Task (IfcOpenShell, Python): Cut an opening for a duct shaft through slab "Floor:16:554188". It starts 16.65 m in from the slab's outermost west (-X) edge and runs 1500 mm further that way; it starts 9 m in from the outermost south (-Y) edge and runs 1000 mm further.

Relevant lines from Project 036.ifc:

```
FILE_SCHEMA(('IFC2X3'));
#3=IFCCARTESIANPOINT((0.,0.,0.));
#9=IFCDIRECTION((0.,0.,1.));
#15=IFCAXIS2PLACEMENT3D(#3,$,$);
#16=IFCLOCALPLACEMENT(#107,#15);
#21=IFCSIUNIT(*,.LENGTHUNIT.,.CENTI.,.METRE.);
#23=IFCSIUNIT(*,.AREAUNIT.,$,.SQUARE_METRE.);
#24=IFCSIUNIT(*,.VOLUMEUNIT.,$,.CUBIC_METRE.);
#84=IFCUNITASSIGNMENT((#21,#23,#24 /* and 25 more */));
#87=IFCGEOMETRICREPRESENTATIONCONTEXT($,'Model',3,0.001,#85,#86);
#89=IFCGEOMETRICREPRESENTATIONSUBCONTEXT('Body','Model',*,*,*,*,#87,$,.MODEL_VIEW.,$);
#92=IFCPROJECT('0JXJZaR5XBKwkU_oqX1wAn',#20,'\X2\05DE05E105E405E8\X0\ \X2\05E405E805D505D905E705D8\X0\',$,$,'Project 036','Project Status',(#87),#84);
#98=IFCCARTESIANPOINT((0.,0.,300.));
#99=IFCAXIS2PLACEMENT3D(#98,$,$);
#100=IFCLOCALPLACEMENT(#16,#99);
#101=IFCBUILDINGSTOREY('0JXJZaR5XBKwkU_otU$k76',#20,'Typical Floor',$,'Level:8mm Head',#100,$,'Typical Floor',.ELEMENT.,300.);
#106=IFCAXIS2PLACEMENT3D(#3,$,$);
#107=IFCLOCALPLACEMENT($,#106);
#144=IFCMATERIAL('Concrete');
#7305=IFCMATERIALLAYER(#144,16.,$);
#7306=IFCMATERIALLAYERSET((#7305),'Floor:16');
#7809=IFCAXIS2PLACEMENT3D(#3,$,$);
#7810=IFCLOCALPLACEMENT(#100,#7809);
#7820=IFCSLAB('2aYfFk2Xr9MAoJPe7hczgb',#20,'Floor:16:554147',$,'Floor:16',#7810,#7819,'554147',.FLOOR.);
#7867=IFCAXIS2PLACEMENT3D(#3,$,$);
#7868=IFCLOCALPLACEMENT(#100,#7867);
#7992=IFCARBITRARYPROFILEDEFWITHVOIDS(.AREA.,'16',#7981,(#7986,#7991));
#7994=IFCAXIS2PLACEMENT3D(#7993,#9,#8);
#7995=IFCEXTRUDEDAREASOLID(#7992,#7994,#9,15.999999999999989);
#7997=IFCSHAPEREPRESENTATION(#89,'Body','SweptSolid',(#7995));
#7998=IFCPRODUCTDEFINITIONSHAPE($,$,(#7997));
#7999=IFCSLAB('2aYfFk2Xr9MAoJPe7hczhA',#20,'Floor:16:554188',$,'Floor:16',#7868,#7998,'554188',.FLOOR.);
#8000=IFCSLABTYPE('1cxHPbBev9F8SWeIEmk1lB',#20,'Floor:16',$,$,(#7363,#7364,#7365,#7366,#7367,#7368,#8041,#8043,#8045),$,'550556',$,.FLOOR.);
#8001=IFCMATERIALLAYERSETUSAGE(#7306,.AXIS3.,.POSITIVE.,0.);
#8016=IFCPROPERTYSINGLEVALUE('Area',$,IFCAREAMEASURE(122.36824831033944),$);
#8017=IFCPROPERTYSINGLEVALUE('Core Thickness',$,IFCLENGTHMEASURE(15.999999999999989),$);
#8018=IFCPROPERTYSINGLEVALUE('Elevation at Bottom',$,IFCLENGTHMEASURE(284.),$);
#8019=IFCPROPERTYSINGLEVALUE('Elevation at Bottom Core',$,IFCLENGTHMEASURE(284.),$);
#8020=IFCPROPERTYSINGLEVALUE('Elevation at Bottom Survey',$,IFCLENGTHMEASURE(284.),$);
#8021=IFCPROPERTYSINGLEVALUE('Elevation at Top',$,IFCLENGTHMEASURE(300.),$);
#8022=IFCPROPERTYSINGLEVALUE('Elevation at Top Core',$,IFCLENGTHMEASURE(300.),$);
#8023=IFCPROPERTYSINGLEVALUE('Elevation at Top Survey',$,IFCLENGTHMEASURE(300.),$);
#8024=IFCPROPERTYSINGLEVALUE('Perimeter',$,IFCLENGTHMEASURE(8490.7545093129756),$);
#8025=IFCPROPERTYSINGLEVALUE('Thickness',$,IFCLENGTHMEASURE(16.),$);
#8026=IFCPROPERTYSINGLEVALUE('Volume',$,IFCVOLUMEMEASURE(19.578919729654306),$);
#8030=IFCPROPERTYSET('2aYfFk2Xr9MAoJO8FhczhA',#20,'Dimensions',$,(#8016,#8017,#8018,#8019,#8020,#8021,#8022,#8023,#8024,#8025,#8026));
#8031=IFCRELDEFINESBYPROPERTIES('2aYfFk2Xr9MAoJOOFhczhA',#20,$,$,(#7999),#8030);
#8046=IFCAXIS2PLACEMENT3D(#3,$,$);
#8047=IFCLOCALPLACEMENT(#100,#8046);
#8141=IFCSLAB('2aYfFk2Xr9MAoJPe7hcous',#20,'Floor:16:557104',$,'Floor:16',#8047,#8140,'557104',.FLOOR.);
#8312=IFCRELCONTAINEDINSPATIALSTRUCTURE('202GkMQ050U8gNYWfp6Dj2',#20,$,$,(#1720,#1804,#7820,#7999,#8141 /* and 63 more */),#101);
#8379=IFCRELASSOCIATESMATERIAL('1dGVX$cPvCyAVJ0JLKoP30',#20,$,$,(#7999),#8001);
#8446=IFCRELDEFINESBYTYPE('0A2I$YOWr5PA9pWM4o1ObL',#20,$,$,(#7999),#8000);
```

```python
import numpy as np
import ifcopenshell
import ifcopenshell.api.feature
import ifcopenshell.api.geometry
import ifcopenshell.api.pset
import ifcopenshell.api.root
import ifcopenshell.geom
import ifcopenshell.util.element
import ifcopenshell.util.placement
import ifcopenshell.util.representation
import ifcopenshell.util.shape
import ifcopenshell.util.unit

model = ifcopenshell.open("Project 036.ifc")
unit_scale = ifcopenshell.util.unit.calculate_unit_scale(model)
area_scale = ifcopenshell.util.unit.calculate_unit_scale(model, "AREAUNIT")
volume_scale = ifcopenshell.util.unit.calculate_unit_scale(model, "VOLUMEUNIT")
settings = ifcopenshell.geom.settings()


def volume(element):
    """Net volume in cubic metres, openings subtracted."""
    shape = ifcopenshell.geom.create_shape(settings, element)
    return ifcopenshell.util.shape.get_volume(shape.geometry)


slab = model.by_guid("2aYfFk2Xr9MAoJPe7hczhA")
before = volume(slab)

# Extent in the slab's own axes, in metres. The edges named are its -X and -Y sides.
slab_shape = ifcopenshell.geom.create_shape(settings, slab)
vertices = ifcopenshell.util.shape.get_vertices(slab_shape.geometry)
x_min, y_min, bottom = vertices.min(axis=0)
top = vertices[:, 2].max()

opening = ifcopenshell.api.root.create_entity(model, ifc_class="IfcOpeningElement", name="Duct shaft opening")
context = ifcopenshell.util.representation.get_context(model, "Model", "Body", "MODEL_VIEW")
width, depth = 1.5, 1
outline = [(0.0, 0.0), (width, 0.0), (width, depth), (0.0, depth), (0.0, 0.0)]
# Overshoot both faces by 50 mm so the cut is clean.
shape = ifcopenshell.api.geometry.add_slab_representation(
    model, context=context, depth=top - bottom + 0.1, polyline=outline
)
ifcopenshell.api.geometry.assign_representation(model, product=opening, representation=shape)

matrix = ifcopenshell.util.placement.get_local_placement(slab.ObjectPlacement)
matrix[:, 3] = matrix @ np.append(np.array([x_min + 16.65, y_min + 9, bottom - 0.05]) / unit_scale, 1.0)
ifcopenshell.api.geometry.edit_object_placement(model, product=opening, matrix=matrix, is_si=False)
ifcopenshell.api.feature.add_feature(model, feature=opening, element=slab)

after = volume(slab)

# Update the slab's stored quantities.
pset = model.by_id(ifcopenshell.util.element.get_pset(slab, "Dimensions", should_inherit=False)["id"])
ifcopenshell.api.pset.edit_pset(model, pset=pset, properties={
    "Area": model.create_entity("IfcAreaMeasure", after / (top - bottom) / area_scale),
    "Volume": model.create_entity("IfcVolumeMeasure", after / volume_scale),
})

print(f"slab volume {before:.3f} -> {after:.3f} m3")

model.write("Project 036-out.ifc")
```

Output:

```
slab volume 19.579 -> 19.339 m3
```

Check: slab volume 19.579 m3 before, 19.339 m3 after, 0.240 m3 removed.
